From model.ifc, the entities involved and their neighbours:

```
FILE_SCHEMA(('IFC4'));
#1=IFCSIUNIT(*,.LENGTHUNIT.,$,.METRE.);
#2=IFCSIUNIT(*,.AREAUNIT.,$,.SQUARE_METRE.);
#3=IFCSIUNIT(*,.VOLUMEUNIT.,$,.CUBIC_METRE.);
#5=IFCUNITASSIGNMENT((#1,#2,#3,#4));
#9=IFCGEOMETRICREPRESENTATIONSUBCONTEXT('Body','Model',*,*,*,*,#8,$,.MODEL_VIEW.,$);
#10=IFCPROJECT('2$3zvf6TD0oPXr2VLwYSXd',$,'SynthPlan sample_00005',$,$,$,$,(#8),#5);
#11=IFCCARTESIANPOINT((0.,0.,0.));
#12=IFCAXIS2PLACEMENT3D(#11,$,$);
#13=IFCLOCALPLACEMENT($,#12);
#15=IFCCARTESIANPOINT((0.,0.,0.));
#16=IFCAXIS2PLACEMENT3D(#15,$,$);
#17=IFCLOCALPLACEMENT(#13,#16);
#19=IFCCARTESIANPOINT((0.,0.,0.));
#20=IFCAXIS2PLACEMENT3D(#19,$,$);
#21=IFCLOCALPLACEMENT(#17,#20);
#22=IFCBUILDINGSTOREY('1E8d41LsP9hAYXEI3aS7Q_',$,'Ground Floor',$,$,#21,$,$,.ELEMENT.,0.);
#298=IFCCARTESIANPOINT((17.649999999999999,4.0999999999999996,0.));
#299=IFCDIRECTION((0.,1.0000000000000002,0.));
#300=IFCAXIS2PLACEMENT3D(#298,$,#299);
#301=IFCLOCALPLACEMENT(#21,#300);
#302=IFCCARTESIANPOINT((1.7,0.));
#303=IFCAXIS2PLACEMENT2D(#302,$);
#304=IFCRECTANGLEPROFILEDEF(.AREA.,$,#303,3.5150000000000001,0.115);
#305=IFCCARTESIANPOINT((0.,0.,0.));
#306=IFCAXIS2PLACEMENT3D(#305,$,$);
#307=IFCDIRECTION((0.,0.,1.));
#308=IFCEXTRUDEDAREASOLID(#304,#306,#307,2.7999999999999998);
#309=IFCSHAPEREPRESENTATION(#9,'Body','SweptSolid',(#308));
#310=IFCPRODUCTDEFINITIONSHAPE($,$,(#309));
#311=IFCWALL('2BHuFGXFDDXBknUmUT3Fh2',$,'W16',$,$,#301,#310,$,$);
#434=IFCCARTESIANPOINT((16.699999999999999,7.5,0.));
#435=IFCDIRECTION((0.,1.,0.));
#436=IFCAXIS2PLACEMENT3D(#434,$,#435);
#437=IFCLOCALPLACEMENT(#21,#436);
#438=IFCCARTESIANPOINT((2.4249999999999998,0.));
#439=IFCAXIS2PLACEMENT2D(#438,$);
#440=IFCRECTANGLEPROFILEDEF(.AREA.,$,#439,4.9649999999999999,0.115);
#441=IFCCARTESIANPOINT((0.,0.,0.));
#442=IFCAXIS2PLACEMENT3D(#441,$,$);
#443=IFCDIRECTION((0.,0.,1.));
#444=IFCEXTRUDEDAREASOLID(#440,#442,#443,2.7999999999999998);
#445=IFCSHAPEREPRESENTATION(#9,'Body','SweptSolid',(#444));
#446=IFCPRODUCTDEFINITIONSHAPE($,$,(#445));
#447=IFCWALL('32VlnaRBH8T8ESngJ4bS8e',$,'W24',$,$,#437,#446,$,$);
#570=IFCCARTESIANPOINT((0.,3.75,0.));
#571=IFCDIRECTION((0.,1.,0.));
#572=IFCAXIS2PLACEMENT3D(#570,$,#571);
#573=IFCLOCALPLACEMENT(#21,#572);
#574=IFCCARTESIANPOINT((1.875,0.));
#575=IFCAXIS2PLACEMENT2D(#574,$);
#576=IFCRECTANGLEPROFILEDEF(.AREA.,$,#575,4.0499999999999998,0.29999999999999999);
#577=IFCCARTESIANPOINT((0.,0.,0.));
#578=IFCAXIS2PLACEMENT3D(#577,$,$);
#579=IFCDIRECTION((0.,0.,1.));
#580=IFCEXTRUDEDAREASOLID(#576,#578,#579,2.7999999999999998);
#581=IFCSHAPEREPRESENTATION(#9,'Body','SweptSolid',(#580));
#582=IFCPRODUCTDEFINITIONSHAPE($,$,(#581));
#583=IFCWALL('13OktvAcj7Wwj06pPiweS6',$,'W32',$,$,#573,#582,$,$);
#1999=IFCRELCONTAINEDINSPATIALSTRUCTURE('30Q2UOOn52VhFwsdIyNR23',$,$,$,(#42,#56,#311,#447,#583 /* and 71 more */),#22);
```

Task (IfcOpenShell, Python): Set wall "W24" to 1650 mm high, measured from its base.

```python
import ifcopenshell
import ifcopenshell.geom
import ifcopenshell.util.representation
import ifcopenshell.util.shape
import ifcopenshell.util.unit

model = ifcopenshell.open("model.ifc")
unit_scale = ifcopenshell.util.unit.calculate_unit_scale(model)
settings = ifcopenshell.geom.settings()


def volume(element):
    """Net volume in cubic metres, openings subtracted."""
    shape = ifcopenshell.geom.create_shape(settings, element)
    return ifcopenshell.util.shape.get_volume(shape.geometry)


wall = model.by_guid("32VlnaRBH8T8ESngJ4bS8e")
before = volume(wall)

body = ifcopenshell.util.representation.get_representation(wall, "Model", "Body")
solid = body.Items[0]
old_height = solid.Depth
solid.Depth = 1.65 / unit_scale
after = volume(wall)

print(f"height {old_height:g} -> {solid.Depth:g}, volume {before:.3f} -> {after:.3f} m3")

model.write("model_edited.ifc")
```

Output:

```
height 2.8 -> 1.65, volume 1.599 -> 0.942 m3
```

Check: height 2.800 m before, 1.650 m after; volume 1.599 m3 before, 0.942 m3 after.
